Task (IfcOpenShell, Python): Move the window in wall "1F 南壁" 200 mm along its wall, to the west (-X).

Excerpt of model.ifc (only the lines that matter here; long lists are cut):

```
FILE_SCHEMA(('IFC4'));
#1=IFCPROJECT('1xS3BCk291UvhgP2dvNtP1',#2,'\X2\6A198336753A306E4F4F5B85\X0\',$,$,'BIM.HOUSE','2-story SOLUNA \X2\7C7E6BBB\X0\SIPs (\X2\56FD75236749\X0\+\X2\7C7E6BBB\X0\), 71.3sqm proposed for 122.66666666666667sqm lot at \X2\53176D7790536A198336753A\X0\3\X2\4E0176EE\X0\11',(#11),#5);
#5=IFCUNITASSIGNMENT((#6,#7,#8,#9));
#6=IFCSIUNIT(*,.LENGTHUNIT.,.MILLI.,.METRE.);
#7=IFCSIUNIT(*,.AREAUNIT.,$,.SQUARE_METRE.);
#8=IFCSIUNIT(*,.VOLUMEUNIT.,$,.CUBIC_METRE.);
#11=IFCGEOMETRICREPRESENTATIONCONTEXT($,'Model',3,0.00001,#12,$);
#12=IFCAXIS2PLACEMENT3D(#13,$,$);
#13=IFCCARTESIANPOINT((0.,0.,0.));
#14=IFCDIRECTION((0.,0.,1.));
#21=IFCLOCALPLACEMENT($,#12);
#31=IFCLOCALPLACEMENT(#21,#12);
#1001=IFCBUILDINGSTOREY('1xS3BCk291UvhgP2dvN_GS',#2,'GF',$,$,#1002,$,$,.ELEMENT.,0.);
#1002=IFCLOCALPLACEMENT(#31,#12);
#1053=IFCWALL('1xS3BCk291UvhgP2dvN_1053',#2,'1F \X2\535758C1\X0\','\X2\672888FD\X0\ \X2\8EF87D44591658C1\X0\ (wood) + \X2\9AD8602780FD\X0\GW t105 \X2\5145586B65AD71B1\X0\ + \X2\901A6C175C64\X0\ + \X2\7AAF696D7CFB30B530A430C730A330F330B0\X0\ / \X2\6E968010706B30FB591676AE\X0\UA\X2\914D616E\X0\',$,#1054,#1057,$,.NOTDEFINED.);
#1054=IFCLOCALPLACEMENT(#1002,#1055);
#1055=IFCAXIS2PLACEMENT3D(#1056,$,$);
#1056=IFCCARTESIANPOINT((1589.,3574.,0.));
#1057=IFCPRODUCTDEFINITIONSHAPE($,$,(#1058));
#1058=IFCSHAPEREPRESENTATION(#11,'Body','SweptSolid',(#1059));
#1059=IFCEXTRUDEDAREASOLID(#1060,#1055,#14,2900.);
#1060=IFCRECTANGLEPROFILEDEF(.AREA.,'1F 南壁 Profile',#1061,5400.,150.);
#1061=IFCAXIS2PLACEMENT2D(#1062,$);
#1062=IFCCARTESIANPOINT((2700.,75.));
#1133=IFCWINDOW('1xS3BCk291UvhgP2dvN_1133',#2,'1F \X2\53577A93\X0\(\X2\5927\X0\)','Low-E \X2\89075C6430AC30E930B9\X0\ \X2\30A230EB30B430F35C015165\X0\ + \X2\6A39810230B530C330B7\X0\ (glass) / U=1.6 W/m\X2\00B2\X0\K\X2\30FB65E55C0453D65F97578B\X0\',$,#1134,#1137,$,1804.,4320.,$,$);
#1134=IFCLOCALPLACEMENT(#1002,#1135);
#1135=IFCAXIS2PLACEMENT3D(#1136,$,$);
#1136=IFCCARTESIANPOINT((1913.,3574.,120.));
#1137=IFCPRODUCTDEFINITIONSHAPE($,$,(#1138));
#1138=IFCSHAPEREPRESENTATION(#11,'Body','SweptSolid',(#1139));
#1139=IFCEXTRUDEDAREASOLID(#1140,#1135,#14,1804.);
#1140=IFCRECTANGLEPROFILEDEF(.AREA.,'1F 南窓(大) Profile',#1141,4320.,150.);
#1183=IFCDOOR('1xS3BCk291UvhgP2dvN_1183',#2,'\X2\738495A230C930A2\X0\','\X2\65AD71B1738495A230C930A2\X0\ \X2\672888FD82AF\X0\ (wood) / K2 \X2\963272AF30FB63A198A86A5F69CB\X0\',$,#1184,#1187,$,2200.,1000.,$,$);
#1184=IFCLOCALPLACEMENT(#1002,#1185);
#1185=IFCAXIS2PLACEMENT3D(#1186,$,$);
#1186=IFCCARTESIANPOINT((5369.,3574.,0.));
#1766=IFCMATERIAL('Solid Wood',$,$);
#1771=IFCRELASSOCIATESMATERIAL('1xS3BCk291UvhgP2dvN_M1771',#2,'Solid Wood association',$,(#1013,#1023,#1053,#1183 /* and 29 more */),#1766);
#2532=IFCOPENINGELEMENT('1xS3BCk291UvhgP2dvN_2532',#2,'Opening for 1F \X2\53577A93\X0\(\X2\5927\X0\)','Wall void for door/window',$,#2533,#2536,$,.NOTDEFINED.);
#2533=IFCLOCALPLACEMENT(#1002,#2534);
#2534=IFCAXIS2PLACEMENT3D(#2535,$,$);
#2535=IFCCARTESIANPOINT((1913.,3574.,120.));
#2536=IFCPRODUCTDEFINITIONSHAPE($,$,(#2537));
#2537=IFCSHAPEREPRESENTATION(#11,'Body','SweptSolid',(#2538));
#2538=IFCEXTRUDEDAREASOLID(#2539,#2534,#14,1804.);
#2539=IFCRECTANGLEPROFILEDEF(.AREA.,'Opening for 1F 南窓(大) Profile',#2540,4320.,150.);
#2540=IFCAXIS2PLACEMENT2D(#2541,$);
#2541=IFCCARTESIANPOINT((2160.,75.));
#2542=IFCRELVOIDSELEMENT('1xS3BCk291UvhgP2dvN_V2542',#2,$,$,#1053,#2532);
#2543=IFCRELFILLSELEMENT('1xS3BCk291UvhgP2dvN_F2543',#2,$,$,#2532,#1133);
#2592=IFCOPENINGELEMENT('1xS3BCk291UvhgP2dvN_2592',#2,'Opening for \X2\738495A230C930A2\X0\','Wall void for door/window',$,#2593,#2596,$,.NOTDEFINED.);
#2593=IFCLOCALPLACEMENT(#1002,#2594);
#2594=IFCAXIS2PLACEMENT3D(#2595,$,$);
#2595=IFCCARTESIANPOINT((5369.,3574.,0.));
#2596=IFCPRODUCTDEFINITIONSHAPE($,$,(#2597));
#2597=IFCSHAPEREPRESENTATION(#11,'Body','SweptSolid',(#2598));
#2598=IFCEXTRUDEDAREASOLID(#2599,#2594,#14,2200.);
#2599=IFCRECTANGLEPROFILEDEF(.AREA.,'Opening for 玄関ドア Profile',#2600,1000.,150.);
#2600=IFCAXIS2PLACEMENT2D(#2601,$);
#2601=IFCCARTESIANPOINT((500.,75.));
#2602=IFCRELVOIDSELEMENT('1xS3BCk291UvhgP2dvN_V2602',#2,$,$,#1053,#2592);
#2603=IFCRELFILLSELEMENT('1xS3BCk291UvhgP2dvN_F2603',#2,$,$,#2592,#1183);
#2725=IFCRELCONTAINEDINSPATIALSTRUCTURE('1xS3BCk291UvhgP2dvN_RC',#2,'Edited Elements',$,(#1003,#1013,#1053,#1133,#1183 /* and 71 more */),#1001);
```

```python
import ifcopenshell
import ifcopenshell.api.geometry
import ifcopenshell.util.placement
import ifcopenshell.util.unit

model = ifcopenshell.open("model.ifc")
unit_scale = ifcopenshell.util.unit.calculate_unit_scale(model)

window = model.by_guid("1xS3BCk291UvhgP2dvN_1133")
opening = window.FillsVoids[0].RelatingOpeningElement
wall = opening.VoidsElements[0].RelatingBuildingElement

wall_matrix = ifcopenshell.util.placement.get_local_placement(wall.ObjectPlacement)
shift = wall_matrix[:3, 0] * -0.2 / unit_scale
before = ifcopenshell.util.placement.get_local_placement(window.ObjectPlacement)[:3, 3].copy()

# The window is not placed relative to its opening, so move both.
for product in (opening, window):
    matrix = ifcopenshell.util.placement.get_local_placement(product.ObjectPlacement)
    matrix[:3, 3] += shift
    ifcopenshell.api.geometry.edit_object_placement(model, product=product, matrix=matrix, is_si=False)

after = ifcopenshell.util.placement.get_local_placement(window.ObjectPlacement)[:3, 3]
print("window moved by", (after - before).round(3) + 0.0)

model.write("model_edited.ifc")
```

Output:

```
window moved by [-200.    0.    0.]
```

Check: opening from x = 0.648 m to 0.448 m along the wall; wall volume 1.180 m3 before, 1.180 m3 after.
